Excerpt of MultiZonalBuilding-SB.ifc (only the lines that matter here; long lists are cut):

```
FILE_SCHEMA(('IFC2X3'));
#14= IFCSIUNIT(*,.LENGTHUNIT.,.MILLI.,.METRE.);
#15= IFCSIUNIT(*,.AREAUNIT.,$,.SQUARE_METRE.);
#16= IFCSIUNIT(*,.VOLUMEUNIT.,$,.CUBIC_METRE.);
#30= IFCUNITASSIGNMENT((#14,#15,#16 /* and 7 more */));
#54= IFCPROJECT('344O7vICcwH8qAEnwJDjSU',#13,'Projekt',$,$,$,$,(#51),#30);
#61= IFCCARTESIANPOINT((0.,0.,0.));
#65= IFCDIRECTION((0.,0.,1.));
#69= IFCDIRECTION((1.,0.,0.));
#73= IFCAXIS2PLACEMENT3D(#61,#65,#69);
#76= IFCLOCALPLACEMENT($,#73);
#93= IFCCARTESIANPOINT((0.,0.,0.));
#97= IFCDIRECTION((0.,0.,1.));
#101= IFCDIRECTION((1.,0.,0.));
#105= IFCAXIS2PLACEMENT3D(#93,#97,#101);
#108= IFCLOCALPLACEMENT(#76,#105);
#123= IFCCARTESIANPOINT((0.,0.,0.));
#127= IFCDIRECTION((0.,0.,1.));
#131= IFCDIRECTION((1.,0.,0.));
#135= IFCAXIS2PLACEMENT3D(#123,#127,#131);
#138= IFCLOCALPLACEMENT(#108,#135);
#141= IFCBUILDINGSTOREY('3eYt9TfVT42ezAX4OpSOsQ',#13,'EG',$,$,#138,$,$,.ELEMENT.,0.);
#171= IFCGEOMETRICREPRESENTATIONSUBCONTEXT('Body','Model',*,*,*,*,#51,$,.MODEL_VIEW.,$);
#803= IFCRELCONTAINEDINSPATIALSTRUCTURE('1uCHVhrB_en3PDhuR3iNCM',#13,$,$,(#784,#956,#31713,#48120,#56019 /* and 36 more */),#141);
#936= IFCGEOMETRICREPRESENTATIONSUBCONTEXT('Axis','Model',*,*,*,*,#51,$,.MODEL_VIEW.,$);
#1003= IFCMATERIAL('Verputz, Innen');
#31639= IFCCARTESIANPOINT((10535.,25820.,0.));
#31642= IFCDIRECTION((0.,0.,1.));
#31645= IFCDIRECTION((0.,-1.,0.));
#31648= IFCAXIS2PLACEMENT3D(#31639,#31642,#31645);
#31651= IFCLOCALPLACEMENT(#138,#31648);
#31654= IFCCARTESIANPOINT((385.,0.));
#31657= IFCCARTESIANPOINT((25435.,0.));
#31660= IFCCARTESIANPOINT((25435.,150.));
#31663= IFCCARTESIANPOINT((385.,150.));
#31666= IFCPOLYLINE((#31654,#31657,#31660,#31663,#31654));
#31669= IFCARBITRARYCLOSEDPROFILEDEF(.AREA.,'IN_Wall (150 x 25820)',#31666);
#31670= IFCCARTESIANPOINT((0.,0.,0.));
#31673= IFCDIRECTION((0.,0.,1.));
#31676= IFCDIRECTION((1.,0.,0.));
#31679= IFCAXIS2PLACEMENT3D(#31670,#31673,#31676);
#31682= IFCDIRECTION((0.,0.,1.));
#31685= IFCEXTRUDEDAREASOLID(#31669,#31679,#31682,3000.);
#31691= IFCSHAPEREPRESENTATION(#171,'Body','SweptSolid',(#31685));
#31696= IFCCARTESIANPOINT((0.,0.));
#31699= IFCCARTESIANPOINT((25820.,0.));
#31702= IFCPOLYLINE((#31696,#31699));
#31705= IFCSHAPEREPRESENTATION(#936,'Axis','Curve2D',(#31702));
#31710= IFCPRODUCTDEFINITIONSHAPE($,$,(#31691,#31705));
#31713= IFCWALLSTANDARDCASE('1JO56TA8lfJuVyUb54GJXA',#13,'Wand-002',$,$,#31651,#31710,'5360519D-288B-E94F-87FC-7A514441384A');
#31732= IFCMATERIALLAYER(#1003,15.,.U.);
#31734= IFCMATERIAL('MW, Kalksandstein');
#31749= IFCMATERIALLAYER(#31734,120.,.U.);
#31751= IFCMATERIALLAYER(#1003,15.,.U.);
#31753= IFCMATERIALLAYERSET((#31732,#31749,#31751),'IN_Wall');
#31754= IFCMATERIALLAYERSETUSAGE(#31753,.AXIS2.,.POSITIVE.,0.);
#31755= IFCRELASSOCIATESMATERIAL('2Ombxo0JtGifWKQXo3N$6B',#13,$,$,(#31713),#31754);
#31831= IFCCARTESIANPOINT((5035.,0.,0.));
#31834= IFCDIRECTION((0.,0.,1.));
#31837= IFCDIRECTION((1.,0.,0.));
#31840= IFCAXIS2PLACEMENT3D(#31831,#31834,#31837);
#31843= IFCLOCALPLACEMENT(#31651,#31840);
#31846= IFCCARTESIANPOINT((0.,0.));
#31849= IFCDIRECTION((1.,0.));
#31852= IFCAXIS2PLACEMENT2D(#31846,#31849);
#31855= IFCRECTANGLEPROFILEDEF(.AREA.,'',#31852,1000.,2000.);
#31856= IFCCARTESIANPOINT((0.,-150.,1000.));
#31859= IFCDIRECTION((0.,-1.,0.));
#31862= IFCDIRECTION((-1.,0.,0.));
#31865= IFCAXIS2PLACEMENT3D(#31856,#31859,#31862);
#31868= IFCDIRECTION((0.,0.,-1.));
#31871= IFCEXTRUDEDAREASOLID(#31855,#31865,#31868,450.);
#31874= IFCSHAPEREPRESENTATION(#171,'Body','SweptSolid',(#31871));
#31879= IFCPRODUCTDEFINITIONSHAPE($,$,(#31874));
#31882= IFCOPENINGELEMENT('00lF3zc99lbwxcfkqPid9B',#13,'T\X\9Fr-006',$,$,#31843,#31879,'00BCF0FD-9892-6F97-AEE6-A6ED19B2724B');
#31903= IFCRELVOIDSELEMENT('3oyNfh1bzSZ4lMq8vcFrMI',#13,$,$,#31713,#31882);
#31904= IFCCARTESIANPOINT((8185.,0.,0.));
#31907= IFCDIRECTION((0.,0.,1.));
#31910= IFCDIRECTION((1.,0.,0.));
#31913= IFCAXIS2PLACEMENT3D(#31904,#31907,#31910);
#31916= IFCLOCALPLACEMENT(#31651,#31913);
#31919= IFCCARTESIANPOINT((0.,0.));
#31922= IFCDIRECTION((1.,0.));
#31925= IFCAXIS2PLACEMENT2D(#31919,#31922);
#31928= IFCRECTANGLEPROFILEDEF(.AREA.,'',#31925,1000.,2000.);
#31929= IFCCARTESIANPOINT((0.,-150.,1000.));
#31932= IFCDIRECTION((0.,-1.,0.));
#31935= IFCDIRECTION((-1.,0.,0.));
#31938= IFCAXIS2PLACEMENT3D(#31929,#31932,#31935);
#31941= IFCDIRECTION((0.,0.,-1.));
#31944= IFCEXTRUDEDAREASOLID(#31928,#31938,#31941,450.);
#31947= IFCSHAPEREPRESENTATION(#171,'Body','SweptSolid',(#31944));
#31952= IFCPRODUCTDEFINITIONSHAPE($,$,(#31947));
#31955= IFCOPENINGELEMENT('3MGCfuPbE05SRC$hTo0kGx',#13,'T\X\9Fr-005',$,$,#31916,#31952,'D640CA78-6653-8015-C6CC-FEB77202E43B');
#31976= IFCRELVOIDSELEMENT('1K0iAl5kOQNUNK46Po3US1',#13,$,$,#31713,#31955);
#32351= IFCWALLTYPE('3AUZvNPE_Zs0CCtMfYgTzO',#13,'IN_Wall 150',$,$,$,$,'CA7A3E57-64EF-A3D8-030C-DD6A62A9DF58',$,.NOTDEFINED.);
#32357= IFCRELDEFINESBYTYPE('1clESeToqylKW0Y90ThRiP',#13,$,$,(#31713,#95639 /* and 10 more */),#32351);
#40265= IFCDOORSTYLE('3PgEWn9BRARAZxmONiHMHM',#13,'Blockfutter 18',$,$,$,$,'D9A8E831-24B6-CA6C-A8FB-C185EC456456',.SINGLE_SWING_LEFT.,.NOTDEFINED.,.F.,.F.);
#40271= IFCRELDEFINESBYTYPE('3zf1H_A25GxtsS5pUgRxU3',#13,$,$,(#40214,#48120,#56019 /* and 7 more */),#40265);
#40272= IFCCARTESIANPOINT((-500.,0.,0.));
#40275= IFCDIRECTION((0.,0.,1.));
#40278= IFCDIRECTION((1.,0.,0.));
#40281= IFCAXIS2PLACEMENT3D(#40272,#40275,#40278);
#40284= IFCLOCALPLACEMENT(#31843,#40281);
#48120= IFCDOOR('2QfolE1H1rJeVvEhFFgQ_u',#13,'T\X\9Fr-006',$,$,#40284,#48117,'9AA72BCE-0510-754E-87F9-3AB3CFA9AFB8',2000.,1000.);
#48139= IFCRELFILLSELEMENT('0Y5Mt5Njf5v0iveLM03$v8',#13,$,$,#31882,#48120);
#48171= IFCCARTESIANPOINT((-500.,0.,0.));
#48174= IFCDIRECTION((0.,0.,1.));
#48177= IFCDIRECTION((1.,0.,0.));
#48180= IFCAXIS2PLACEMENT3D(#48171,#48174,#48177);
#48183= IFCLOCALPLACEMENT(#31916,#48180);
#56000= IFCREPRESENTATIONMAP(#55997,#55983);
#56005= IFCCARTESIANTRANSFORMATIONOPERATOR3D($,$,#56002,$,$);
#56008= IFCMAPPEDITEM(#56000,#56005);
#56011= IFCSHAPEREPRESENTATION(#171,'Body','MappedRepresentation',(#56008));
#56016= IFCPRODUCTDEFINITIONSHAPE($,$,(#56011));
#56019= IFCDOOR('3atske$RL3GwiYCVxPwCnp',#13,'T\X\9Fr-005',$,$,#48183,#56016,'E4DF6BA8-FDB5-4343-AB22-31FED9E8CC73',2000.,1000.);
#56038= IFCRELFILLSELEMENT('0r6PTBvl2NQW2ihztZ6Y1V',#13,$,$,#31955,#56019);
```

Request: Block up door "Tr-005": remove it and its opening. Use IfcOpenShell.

```python
import ifcopenshell
import ifcopenshell.api.feature
import ifcopenshell.api.root
import ifcopenshell.geom
import ifcopenshell.util.shape

model = ifcopenshell.open("MultiZonalBuilding-SB.ifc")
settings = ifcopenshell.geom.settings()


def volume(element):
    """Net volume in cubic metres, openings subtracted."""
    shape = ifcopenshell.geom.create_shape(settings, element)
    return ifcopenshell.util.shape.get_volume(shape.geometry)


door = model.by_id(56019)
opening = door.FillsVoids[0].RelatingOpeningElement
wall = opening.VoidsElements[0].RelatingBuildingElement
before = volume(wall)

ifcopenshell.api.root.remove_product(model, product=door)
ifcopenshell.api.feature.remove_feature(model, feature=opening)

after = volume(wall)

print(f"wall volume {before:.3f} -> {after:.3f} m3")

model.write("MultiZonalBuilding-SB_rev.ifc")
```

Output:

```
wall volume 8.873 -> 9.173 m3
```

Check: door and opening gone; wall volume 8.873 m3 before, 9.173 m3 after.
